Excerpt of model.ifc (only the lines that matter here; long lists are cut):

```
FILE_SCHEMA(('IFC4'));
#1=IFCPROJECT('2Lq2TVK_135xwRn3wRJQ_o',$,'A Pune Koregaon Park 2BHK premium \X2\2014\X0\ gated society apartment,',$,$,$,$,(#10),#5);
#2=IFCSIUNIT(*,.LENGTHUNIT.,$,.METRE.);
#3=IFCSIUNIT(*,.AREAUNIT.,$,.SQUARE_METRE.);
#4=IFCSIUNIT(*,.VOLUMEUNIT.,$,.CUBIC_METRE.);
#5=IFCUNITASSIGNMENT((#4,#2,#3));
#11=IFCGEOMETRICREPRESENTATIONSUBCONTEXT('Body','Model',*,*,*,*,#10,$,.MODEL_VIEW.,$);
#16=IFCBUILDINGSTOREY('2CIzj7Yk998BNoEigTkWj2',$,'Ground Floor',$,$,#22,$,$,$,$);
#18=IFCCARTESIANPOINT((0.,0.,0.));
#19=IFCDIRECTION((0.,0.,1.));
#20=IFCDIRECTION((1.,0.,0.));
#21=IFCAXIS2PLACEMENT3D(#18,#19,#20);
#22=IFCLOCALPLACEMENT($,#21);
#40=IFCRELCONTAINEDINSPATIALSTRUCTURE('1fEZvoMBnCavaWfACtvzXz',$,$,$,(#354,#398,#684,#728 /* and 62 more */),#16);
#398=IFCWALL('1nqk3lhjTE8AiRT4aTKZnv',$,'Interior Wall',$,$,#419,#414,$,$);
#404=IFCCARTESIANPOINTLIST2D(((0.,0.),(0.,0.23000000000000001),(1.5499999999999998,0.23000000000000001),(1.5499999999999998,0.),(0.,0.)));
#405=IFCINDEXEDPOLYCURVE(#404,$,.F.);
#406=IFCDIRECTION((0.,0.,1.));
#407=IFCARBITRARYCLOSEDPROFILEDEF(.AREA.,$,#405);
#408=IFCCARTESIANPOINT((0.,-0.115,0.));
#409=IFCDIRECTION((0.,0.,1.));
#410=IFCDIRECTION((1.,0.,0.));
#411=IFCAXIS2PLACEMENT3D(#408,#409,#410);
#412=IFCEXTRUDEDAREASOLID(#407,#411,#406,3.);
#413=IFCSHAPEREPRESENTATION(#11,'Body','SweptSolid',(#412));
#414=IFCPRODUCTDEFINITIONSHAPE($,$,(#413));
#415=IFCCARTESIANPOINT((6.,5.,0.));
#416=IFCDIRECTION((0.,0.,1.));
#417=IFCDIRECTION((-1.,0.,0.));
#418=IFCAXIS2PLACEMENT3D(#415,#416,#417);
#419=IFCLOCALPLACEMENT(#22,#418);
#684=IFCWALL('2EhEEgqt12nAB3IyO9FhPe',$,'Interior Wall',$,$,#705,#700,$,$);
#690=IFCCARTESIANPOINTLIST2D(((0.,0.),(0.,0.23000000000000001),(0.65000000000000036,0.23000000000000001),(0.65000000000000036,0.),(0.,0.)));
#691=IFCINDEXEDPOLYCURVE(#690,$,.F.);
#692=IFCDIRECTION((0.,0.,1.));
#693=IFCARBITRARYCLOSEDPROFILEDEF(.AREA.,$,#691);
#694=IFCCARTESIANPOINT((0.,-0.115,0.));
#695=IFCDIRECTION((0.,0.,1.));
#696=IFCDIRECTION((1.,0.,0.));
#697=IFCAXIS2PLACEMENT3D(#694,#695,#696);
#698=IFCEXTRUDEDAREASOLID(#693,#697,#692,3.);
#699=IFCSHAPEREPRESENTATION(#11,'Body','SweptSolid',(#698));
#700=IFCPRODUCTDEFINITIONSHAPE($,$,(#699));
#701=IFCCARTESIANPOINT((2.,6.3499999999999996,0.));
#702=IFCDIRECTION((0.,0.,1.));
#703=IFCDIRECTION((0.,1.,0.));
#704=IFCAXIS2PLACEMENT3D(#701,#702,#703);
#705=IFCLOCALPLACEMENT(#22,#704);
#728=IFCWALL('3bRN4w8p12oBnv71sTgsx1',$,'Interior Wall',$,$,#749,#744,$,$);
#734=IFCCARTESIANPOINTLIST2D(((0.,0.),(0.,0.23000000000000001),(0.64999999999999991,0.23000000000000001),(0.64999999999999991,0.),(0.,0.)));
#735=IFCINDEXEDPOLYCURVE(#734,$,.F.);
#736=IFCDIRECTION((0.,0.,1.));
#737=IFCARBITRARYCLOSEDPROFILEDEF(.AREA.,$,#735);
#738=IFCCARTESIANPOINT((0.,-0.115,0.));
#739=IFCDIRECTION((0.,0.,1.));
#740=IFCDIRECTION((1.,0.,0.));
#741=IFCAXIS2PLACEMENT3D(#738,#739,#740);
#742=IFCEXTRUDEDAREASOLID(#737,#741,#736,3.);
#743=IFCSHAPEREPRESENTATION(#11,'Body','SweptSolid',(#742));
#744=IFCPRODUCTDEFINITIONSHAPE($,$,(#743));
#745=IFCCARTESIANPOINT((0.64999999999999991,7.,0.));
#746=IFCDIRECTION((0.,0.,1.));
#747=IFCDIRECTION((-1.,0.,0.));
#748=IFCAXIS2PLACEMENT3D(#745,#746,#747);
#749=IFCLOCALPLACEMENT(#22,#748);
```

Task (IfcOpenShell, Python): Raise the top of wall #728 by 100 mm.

```python
import ifcopenshell
import ifcopenshell.geom
import ifcopenshell.util.representation
import ifcopenshell.util.shape

model = ifcopenshell.open("model.ifc")
settings = ifcopenshell.geom.settings()


def volume(element):
    """Net volume in cubic metres, openings subtracted."""
    shape = ifcopenshell.geom.create_shape(settings, element)
    return ifcopenshell.util.shape.get_volume(shape.geometry)


wall = model.by_id(728)
before = volume(wall)

body = ifcopenshell.util.representation.get_representation(wall, "Model", "Body")
solid = body.Items[0]
old_height = solid.Depth
solid.Depth += 0.1
after = volume(wall)

print(f"height {old_height:g} -> {solid.Depth:g}, volume {before:.3f} -> {after:.3f} m3")

model.write("model_rev.ifc")
```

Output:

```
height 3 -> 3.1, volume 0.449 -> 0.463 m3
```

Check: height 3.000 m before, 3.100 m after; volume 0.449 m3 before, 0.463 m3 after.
